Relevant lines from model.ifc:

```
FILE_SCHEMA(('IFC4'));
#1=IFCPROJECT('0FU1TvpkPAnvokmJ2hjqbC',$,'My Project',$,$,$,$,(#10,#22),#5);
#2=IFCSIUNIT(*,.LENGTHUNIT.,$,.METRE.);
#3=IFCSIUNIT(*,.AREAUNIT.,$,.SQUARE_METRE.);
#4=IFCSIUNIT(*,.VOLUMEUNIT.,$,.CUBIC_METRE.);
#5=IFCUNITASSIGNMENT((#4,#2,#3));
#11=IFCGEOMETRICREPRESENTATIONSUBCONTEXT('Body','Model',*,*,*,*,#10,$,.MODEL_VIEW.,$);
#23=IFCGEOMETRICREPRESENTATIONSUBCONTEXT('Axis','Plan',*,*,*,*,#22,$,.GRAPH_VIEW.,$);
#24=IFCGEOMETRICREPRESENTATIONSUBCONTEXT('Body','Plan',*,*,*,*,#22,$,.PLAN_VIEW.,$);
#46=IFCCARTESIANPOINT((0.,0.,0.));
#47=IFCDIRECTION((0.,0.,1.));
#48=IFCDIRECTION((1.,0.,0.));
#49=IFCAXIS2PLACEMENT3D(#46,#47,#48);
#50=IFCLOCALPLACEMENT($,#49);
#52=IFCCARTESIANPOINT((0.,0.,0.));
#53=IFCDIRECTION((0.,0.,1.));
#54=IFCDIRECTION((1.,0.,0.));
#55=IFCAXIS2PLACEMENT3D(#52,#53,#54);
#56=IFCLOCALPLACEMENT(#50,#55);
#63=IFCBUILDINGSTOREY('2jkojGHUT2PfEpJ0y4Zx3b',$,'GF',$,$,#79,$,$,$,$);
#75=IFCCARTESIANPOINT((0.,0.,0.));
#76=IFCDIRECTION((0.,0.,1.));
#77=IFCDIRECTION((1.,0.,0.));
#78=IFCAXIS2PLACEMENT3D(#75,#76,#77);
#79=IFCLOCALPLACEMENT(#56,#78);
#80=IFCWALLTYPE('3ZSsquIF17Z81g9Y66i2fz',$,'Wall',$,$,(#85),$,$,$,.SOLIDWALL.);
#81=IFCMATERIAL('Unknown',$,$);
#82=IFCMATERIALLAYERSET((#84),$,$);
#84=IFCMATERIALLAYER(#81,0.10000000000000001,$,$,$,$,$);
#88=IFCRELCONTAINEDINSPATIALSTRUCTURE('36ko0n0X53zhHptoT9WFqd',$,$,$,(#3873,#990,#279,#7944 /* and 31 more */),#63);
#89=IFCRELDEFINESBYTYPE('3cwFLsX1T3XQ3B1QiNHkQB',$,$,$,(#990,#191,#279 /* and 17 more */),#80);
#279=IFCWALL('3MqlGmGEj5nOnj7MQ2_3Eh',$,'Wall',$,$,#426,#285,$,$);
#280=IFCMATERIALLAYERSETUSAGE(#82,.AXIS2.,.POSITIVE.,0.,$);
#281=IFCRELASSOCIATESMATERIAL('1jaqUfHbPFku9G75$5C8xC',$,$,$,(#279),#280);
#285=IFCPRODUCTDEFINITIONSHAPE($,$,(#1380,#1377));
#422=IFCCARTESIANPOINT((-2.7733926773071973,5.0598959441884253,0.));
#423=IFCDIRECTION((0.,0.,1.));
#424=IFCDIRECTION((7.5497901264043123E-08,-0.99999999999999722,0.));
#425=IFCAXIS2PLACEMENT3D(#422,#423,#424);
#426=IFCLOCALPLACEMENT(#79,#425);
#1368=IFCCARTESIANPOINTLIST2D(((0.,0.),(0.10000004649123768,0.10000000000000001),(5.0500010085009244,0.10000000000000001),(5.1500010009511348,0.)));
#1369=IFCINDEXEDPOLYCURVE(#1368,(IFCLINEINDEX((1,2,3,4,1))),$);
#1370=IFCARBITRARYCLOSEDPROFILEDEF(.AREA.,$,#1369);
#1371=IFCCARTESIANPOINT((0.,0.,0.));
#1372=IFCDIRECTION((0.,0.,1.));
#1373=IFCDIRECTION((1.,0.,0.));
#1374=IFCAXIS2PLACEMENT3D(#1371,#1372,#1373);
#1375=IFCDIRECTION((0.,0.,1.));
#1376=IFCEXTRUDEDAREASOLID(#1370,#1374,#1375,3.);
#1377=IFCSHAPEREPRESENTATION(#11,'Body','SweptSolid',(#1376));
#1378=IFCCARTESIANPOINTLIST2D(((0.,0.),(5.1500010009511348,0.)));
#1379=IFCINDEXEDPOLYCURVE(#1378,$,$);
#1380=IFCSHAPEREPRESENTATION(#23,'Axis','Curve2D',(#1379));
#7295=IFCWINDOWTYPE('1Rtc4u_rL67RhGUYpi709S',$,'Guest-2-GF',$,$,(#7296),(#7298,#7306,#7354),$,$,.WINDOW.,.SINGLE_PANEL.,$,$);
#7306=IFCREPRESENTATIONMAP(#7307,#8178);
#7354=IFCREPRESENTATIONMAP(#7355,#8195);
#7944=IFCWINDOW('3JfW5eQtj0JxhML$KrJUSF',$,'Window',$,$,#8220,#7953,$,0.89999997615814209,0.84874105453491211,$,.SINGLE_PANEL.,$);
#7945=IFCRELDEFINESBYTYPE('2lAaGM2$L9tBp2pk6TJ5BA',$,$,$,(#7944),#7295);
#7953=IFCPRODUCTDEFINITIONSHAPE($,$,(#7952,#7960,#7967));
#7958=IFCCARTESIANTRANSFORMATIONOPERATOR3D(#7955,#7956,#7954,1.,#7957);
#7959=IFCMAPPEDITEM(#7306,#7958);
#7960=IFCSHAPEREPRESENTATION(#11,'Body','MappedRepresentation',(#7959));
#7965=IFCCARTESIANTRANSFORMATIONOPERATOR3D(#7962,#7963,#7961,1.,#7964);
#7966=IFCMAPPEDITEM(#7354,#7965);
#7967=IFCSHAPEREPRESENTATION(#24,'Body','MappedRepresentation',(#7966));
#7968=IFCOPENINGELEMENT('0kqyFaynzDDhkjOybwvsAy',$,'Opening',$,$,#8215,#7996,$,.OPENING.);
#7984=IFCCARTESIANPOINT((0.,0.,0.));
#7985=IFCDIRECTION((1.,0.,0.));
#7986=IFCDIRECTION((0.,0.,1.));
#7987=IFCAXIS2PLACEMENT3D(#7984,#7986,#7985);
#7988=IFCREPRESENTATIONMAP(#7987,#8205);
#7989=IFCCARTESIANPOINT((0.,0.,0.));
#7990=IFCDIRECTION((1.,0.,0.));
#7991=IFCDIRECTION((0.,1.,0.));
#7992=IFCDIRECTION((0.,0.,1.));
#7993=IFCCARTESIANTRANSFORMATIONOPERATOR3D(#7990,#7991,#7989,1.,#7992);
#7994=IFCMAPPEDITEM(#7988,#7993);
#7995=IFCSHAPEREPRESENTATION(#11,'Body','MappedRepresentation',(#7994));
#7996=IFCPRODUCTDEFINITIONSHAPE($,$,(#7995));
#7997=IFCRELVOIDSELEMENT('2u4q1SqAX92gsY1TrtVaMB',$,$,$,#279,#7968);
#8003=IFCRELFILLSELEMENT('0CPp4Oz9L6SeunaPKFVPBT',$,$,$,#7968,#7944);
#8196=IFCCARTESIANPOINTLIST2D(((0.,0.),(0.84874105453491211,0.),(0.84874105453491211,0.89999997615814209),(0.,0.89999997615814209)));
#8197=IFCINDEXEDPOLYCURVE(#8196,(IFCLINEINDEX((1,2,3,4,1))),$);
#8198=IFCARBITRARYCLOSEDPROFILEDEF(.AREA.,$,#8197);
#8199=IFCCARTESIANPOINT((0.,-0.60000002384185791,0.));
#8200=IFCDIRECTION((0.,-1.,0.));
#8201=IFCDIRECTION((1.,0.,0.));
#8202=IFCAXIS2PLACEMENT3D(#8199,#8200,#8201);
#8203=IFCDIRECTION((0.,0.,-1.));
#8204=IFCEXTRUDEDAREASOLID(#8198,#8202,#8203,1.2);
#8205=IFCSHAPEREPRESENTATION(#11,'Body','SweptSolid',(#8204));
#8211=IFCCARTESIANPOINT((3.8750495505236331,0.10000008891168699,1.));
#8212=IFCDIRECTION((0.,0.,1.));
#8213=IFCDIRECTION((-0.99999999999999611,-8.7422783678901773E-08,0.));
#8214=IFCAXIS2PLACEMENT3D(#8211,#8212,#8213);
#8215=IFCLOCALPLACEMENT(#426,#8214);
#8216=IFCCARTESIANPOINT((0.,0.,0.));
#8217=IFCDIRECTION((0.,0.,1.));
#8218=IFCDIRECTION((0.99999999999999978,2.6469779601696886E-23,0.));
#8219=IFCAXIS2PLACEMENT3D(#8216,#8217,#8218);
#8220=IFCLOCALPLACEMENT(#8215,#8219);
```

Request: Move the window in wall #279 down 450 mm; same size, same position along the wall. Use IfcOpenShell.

```python
import numpy as np
import ifcopenshell
import ifcopenshell.api.geometry
import ifcopenshell.util.placement
import ifcopenshell.util.unit

model = ifcopenshell.open("model.ifc")
unit_scale = ifcopenshell.util.unit.calculate_unit_scale(model)

window = model.by_guid("3JfW5eQtj0JxhML$KrJUSF")
opening = window.FillsVoids[0].RelatingOpeningElement
dz = -0.45 / unit_scale

shift = np.array([0.0, 0.0, dz])
# The window is placed relative to its opening, so it follows when the opening moves.
matrix = ifcopenshell.util.placement.get_local_placement(opening.ObjectPlacement)
matrix[:3, 3] += shift
ifcopenshell.api.geometry.edit_object_placement(
    model, product=opening, matrix=matrix, is_si=False, should_transform_children=True
)

print(f"moved by {dz * unit_scale:+.3f} m")

model.write("model-out.ifc")
```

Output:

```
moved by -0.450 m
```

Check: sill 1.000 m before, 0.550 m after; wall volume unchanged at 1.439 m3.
